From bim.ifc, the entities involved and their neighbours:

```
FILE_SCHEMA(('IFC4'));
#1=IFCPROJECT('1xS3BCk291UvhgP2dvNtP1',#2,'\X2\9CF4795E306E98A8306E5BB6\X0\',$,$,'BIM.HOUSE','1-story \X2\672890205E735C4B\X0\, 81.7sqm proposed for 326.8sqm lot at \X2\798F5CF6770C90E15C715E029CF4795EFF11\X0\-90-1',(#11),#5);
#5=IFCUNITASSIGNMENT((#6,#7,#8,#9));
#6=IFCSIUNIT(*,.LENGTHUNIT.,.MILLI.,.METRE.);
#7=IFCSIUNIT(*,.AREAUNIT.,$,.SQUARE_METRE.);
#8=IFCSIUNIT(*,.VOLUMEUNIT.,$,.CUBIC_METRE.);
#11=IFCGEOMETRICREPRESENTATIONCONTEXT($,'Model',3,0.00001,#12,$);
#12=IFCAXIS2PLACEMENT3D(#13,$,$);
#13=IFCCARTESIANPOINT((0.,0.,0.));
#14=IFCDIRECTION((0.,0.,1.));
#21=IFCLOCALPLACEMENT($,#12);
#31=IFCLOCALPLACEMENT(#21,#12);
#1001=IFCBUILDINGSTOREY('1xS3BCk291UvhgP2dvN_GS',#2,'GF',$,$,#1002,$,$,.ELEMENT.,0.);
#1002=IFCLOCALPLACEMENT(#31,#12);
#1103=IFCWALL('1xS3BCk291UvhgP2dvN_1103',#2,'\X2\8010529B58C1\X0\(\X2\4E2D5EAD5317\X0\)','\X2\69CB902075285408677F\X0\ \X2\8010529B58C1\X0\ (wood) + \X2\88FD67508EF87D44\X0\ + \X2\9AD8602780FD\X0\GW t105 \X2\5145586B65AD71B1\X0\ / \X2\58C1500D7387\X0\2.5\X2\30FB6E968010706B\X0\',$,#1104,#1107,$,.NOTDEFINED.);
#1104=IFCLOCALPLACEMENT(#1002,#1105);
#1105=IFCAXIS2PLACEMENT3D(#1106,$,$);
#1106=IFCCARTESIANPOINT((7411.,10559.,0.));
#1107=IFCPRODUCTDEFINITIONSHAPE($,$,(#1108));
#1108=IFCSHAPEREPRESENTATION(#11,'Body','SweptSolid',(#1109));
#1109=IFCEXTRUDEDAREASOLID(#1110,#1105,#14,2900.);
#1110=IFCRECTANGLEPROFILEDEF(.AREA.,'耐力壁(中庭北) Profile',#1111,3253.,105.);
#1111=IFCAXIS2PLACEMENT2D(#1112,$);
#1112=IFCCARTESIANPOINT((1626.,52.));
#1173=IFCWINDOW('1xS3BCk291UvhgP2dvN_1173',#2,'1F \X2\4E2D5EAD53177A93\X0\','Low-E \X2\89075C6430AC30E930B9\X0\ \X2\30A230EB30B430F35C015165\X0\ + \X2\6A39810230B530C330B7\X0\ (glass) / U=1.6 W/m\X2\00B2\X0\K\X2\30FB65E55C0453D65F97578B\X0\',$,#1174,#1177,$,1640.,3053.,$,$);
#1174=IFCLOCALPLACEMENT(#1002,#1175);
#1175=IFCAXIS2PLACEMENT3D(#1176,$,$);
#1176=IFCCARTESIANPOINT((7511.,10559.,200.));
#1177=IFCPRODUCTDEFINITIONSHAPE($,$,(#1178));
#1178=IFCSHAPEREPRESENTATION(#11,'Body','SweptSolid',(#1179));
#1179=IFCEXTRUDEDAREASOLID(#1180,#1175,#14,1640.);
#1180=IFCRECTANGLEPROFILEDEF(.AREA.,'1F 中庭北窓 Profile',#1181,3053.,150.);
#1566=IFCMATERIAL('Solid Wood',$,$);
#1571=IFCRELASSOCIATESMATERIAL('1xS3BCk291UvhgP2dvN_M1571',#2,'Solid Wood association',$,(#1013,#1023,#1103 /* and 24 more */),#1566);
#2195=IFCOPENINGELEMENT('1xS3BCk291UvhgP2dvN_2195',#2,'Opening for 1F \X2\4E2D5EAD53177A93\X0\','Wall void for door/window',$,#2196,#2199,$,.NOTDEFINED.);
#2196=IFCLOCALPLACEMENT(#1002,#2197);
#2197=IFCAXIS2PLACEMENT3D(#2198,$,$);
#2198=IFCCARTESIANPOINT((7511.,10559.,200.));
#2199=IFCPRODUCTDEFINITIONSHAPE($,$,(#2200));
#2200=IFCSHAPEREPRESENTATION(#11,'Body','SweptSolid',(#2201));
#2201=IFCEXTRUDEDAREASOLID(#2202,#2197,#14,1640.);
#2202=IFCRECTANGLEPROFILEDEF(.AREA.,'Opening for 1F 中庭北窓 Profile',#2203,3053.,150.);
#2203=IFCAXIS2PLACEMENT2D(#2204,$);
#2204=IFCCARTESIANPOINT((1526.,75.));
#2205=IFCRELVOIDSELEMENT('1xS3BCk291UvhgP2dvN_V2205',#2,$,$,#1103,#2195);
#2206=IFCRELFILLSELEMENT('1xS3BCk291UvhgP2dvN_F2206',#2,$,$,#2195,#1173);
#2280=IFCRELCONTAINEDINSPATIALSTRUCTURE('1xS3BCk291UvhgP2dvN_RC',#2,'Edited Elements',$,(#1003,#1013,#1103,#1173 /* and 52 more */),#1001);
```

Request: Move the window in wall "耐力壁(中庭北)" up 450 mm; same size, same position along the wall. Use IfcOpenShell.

```python
import numpy as np
import ifcopenshell
import ifcopenshell.api.geometry
import ifcopenshell.util.placement
import ifcopenshell.util.unit

model = ifcopenshell.open("bim.ifc")
unit_scale = ifcopenshell.util.unit.calculate_unit_scale(model)

window = model.by_guid("1xS3BCk291UvhgP2dvN_1173")
opening = window.FillsVoids[0].RelatingOpeningElement
dz = 0.45 / unit_scale

shift = np.array([0.0, 0.0, dz])
# The window is not placed relative to its opening, so move both.
for product in (opening, window):
    matrix = ifcopenshell.util.placement.get_local_placement(product.ObjectPlacement)
    matrix[:3, 3] += shift
    ifcopenshell.api.geometry.edit_object_placement(model, product=product, matrix=matrix, is_si=False)

print(f"moved by {dz * unit_scale:+.3f} m")

model.write("bim_rev.ifc")
```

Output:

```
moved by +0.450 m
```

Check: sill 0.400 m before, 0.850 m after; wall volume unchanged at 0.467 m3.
